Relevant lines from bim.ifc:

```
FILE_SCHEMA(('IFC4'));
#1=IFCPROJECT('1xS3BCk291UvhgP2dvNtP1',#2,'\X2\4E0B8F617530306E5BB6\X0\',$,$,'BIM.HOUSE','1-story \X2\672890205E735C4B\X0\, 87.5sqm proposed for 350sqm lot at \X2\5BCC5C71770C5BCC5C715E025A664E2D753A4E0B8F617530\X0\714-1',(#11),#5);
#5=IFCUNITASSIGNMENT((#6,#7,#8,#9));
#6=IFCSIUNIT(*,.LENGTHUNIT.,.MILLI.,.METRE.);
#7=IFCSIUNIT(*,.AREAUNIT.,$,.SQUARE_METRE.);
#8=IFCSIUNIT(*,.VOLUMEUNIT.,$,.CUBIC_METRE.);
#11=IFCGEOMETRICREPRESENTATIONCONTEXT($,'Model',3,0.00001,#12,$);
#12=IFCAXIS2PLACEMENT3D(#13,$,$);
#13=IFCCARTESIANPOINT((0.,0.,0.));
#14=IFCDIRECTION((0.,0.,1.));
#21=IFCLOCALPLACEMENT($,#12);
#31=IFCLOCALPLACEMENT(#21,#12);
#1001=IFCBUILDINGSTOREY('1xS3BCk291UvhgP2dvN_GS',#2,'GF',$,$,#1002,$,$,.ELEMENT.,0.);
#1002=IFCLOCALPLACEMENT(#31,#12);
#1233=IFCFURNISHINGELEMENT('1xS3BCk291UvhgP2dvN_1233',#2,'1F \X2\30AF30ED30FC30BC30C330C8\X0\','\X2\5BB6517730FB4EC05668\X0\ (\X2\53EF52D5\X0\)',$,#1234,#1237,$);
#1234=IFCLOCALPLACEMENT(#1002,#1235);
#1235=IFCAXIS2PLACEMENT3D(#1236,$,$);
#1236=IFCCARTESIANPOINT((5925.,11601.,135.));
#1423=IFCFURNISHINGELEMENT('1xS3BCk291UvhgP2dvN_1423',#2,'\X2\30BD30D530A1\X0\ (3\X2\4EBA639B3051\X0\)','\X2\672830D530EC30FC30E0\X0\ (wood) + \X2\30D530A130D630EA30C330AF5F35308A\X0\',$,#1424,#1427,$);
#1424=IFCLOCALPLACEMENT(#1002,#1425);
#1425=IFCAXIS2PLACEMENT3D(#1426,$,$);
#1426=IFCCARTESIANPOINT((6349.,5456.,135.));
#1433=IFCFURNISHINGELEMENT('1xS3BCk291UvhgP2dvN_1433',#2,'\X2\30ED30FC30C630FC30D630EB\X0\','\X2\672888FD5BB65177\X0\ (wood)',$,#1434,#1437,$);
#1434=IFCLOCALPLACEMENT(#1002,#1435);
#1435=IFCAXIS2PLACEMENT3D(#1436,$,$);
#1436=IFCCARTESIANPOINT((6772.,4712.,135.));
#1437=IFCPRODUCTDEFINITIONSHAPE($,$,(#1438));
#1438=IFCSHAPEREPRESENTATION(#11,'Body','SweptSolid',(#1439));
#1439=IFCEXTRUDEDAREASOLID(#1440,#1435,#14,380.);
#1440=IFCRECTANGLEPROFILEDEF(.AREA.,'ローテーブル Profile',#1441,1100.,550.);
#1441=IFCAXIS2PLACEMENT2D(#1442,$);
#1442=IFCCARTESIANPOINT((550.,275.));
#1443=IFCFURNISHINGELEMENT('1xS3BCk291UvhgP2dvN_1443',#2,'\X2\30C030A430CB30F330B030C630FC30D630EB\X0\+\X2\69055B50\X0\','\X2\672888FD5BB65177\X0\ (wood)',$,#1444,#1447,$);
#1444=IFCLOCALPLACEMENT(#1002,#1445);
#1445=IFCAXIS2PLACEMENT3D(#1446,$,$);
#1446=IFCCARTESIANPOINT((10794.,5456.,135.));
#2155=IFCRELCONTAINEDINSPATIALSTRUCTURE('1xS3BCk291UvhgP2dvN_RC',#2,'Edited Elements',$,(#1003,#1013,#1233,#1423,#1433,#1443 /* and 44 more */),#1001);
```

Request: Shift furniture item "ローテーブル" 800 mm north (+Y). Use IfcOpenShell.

```python
import ifcopenshell
import ifcopenshell.api.geometry
import ifcopenshell.util.placement

model = ifcopenshell.open("bim.ifc")

item = model.by_id(1433)
matrix = ifcopenshell.util.placement.get_local_placement(item.ObjectPlacement)
matrix[1, 3] += 800.0
ifcopenshell.api.geometry.edit_object_placement(model, product=item, matrix=matrix, is_si=False)

print(ifcopenshell.util.placement.get_local_placement(item.ObjectPlacement).round(3) + 0.0)

model.write("bim_v2.ifc")
```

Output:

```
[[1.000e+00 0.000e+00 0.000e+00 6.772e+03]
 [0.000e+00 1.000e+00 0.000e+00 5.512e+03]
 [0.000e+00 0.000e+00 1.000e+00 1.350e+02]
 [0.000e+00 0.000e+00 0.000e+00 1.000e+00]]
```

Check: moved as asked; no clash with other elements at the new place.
